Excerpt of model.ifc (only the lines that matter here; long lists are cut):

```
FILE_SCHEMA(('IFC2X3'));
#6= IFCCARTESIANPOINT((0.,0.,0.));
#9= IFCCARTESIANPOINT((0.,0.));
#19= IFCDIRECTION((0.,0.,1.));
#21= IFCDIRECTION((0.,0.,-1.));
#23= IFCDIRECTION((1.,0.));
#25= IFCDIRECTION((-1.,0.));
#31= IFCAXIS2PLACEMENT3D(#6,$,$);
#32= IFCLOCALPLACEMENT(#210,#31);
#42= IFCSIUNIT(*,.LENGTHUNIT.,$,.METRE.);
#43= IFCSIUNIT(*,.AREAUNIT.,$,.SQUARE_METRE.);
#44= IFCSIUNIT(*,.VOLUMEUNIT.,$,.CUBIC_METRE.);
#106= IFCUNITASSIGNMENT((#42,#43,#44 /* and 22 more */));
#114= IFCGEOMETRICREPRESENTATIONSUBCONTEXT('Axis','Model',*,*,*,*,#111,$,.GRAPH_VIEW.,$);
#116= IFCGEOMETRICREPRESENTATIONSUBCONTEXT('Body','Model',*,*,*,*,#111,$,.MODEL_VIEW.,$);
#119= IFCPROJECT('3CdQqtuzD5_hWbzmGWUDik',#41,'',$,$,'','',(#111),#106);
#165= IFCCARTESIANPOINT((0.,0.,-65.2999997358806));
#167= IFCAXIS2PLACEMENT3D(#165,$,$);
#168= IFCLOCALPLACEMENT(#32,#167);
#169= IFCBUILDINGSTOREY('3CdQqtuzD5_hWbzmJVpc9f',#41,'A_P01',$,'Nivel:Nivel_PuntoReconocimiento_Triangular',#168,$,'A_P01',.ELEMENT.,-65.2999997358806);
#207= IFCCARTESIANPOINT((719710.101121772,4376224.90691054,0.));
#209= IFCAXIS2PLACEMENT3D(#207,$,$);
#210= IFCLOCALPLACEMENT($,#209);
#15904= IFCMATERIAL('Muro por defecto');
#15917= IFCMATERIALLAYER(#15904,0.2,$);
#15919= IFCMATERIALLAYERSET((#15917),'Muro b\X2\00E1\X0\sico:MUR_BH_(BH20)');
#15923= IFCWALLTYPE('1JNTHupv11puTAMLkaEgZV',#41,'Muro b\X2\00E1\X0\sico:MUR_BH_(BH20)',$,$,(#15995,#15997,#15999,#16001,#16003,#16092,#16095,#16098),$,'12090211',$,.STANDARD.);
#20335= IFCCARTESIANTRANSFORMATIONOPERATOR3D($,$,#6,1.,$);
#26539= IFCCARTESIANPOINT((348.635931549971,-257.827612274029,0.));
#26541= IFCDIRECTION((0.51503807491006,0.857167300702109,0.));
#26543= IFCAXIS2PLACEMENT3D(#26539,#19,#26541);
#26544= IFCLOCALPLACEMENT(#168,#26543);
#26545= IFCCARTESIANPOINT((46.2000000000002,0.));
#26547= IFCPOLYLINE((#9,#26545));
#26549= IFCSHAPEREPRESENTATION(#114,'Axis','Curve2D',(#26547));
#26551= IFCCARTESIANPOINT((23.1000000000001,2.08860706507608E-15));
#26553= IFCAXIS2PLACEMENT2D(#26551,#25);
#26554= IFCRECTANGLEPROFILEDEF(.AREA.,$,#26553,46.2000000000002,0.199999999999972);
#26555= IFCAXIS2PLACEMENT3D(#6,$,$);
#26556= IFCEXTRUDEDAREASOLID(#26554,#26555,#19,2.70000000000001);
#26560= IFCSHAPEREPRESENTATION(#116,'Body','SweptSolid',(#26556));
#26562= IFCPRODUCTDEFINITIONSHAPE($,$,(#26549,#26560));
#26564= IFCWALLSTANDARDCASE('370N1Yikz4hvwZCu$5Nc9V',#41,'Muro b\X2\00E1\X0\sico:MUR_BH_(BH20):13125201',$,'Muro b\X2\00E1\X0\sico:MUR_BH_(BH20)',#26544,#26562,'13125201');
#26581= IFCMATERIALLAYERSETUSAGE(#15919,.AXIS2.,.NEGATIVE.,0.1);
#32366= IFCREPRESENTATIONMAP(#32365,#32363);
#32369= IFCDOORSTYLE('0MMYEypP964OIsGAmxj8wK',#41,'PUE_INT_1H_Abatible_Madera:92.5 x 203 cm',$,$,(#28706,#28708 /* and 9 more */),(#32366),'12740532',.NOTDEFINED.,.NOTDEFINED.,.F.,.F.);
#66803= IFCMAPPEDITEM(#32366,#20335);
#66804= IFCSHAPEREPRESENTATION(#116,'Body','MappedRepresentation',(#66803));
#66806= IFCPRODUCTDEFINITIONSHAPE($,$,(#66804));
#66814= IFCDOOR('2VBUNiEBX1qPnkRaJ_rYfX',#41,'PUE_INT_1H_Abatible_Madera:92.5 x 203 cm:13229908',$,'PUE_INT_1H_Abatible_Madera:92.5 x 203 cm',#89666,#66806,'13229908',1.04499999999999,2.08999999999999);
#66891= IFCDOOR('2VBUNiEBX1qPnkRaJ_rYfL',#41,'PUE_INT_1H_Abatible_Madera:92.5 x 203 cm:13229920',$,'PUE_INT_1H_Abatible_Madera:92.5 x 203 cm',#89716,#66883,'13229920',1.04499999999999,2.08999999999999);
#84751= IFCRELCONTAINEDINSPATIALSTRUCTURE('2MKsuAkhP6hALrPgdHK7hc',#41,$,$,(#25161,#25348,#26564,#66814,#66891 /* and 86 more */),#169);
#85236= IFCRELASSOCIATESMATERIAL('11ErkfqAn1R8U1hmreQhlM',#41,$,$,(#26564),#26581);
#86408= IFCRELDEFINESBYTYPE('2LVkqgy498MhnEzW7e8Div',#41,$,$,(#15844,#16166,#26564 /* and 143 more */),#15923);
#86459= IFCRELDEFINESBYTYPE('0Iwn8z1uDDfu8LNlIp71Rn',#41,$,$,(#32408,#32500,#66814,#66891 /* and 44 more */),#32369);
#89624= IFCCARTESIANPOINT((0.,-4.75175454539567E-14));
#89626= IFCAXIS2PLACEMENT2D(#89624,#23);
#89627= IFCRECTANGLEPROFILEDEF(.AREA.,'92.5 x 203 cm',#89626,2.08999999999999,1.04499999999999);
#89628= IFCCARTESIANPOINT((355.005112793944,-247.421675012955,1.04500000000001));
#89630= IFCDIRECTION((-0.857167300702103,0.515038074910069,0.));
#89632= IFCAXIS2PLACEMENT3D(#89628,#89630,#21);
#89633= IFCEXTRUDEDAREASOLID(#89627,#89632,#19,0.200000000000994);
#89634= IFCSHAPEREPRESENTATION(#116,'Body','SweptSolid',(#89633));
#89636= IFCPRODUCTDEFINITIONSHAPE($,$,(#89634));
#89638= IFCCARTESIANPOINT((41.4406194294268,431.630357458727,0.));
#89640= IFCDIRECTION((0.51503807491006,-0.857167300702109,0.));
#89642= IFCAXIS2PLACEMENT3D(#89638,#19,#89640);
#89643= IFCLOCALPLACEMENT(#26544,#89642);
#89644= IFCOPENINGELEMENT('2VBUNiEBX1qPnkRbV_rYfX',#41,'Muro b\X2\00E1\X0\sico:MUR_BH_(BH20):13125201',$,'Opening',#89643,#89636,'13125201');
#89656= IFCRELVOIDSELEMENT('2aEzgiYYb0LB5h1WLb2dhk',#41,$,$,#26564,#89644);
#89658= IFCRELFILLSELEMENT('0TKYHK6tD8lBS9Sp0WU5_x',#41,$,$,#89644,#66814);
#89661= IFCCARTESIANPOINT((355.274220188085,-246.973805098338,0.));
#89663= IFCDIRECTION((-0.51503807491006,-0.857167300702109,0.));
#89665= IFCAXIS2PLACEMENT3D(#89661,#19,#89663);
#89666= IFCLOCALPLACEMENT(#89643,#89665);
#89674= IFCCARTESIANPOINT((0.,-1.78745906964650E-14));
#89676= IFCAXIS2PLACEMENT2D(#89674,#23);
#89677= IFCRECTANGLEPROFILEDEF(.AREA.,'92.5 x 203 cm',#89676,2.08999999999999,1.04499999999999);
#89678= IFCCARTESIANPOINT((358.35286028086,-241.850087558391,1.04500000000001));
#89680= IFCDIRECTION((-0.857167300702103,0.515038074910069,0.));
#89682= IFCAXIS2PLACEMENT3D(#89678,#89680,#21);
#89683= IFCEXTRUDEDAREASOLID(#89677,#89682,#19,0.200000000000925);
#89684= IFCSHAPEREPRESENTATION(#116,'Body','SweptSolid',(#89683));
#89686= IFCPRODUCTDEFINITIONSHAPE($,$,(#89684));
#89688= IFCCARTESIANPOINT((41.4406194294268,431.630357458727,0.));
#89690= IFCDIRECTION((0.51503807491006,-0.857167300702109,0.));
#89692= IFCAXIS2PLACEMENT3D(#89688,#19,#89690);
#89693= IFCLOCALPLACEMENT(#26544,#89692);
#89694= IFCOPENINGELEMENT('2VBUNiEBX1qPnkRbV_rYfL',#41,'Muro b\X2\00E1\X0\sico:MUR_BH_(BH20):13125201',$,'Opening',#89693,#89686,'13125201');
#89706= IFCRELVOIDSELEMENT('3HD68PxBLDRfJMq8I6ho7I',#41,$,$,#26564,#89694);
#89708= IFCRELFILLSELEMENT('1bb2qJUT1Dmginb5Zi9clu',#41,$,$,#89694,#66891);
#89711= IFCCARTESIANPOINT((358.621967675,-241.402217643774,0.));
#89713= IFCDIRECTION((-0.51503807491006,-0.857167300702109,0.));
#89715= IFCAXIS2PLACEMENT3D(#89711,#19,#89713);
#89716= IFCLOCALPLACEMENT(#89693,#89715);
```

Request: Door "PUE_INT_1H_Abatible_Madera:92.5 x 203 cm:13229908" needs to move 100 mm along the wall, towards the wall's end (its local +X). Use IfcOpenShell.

```python
import ifcopenshell
import ifcopenshell.api.geometry
import ifcopenshell.util.placement

model = ifcopenshell.open("model.ifc")

door = model.by_id(66814)
opening = door.FillsVoids[0].RelatingOpeningElement
wall = opening.VoidsElements[0].RelatingBuildingElement

wall_matrix = ifcopenshell.util.placement.get_local_placement(wall.ObjectPlacement)
shift = wall_matrix[:3, 0] * 0.1
before = ifcopenshell.util.placement.get_local_placement(door.ObjectPlacement)[:3, 3].copy()

# The door is placed relative to its opening, so it follows when the opening moves.
matrix = ifcopenshell.util.placement.get_local_placement(opening.ObjectPlacement)
matrix[:3, 3] += shift
ifcopenshell.api.geometry.edit_object_placement(
    model, product=opening, matrix=matrix, is_si=False, should_transform_children=True
)

after = ifcopenshell.util.placement.get_local_placement(door.ObjectPlacement)[:3, 3]
print("door moved by", (after - before).round(3) + 0.0)

model.write("model-out.ifc")
```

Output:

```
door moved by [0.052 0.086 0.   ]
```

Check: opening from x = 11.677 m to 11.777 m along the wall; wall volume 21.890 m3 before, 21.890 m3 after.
